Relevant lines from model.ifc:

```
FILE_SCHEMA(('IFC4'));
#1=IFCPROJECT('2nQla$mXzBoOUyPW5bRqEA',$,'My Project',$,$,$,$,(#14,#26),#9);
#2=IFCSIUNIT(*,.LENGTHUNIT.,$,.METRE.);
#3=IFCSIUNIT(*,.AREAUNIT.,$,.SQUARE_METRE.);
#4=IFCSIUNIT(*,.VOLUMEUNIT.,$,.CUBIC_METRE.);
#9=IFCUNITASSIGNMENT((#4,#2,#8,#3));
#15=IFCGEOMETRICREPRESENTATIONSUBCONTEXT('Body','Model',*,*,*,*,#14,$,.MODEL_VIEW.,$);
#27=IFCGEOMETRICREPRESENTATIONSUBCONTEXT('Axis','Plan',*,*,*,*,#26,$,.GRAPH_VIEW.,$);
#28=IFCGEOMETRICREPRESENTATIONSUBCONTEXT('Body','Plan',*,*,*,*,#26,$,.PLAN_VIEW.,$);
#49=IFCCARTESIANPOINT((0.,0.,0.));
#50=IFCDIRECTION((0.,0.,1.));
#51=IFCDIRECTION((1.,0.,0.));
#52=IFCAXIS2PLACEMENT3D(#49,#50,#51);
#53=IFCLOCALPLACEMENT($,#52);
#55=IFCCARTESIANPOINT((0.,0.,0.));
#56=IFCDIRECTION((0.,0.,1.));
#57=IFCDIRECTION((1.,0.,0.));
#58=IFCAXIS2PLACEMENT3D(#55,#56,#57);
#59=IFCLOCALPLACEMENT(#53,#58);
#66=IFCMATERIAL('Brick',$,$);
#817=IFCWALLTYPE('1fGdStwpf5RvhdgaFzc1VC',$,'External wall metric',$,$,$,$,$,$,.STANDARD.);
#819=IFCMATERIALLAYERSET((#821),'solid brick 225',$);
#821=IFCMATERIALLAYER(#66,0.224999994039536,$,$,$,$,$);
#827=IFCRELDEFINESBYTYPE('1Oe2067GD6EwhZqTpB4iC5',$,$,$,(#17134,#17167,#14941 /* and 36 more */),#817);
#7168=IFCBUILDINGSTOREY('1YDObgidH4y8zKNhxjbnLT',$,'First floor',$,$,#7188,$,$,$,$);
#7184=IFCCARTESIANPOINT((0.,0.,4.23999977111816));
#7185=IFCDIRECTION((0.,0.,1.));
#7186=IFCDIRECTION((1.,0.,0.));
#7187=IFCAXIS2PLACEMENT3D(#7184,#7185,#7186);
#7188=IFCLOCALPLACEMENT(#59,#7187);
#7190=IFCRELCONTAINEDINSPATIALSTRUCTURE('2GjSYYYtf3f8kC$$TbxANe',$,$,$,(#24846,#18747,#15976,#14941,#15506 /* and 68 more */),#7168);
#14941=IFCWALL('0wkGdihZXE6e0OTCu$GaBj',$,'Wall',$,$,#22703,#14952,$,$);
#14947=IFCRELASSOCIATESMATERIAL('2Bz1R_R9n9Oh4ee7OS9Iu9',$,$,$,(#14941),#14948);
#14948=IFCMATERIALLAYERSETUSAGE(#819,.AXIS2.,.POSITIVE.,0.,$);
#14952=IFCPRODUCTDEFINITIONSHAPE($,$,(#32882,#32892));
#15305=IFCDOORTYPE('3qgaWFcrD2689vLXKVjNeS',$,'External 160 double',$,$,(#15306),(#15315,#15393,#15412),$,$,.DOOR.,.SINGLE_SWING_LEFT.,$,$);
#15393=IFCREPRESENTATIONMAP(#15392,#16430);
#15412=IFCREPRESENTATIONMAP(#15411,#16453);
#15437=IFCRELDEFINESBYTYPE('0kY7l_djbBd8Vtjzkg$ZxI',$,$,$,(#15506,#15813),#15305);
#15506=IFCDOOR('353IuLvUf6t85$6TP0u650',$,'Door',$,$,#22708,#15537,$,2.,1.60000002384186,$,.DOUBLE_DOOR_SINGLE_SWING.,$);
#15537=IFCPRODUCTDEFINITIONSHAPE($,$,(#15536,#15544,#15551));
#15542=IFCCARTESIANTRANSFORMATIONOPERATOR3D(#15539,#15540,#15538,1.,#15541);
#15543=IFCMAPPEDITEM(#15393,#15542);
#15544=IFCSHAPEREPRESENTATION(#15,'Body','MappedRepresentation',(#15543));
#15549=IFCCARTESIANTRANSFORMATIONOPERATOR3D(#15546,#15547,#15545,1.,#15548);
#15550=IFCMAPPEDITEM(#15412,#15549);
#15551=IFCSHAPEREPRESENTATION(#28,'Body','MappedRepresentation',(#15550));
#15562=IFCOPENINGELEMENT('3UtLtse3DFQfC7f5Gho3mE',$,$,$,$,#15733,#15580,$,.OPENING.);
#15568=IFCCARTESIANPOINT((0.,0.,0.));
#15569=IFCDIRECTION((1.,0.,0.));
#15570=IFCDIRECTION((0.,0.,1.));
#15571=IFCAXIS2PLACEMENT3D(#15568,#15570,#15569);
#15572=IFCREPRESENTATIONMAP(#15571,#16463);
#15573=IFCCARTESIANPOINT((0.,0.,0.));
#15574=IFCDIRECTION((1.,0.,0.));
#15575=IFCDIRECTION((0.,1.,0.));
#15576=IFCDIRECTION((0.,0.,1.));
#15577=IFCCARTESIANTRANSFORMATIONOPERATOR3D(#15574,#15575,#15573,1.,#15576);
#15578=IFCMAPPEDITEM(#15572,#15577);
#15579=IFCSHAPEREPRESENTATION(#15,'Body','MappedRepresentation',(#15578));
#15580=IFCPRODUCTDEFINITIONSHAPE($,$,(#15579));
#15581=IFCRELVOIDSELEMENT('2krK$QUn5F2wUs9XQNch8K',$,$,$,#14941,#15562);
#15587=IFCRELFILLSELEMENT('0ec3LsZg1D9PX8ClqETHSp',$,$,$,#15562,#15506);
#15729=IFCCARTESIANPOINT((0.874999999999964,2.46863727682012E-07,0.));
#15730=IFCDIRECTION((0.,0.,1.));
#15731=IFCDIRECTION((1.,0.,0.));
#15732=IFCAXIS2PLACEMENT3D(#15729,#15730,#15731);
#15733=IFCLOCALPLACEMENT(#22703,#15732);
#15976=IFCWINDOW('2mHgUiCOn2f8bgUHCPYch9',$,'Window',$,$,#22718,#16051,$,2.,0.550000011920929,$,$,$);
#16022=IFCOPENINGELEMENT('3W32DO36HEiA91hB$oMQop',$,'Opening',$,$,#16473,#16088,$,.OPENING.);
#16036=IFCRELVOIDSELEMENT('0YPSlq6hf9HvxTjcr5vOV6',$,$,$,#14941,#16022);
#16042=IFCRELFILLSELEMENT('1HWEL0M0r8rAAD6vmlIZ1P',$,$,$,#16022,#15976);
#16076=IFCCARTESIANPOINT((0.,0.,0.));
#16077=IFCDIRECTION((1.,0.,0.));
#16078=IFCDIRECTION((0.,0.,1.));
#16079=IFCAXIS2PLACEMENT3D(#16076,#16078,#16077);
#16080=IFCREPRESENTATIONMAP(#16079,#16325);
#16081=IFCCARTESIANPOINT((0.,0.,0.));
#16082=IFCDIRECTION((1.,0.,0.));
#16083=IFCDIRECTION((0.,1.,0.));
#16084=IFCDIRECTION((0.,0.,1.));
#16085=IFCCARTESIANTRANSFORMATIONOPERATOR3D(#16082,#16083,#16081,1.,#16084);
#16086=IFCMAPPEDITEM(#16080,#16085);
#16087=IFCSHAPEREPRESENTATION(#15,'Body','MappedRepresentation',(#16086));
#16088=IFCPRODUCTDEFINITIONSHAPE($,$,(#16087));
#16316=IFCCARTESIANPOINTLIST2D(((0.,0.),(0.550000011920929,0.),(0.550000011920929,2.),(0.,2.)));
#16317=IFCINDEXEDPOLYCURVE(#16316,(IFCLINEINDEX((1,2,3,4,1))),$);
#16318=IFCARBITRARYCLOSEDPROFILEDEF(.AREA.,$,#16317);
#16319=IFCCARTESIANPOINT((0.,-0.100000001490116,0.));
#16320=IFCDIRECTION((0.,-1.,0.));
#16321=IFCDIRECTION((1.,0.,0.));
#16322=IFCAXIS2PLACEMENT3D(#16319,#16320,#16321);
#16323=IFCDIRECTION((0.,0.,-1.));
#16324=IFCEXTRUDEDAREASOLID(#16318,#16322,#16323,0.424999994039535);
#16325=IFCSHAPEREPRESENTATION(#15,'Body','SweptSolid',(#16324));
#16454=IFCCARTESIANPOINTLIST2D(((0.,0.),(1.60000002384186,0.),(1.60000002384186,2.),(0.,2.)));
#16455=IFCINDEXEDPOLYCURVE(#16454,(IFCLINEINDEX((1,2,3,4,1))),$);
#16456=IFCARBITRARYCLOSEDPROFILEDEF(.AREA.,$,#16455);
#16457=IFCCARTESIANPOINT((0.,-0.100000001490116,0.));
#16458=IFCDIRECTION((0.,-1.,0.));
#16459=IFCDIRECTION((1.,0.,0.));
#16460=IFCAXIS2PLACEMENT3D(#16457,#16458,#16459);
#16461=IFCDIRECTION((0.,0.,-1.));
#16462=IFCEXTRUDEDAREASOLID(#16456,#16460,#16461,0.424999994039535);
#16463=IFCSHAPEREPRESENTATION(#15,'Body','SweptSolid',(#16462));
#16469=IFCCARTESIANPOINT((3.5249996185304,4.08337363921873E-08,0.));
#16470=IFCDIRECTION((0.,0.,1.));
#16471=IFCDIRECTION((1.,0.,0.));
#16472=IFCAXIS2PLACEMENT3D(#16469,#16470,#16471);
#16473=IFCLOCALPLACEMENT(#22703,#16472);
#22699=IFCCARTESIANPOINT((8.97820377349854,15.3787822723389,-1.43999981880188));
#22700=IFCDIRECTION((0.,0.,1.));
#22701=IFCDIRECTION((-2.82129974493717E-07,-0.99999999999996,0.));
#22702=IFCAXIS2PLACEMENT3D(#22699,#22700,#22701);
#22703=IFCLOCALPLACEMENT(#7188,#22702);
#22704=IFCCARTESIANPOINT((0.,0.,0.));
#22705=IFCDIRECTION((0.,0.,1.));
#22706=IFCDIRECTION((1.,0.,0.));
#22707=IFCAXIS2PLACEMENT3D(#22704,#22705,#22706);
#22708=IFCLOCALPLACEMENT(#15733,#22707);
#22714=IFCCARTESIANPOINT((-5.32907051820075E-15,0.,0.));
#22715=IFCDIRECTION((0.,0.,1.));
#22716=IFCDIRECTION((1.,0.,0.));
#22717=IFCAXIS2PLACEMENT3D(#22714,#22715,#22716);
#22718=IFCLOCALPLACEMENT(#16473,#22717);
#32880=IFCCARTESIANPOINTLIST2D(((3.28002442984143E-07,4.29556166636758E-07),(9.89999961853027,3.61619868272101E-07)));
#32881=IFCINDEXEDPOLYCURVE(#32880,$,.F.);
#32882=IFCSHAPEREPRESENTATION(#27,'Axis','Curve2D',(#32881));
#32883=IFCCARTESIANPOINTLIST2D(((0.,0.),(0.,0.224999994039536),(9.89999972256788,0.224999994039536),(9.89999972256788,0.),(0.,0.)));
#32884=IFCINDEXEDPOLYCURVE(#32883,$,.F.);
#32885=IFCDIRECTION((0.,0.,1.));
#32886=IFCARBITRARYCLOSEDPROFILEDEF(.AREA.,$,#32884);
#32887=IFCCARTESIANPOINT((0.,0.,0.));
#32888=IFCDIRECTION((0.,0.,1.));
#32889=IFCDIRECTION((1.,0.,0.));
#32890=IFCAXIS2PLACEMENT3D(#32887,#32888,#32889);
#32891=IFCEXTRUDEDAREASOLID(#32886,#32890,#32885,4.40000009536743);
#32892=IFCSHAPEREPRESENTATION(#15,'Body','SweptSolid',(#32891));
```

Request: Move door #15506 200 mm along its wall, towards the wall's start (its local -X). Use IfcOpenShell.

```python
import ifcopenshell
import ifcopenshell.api.geometry
import ifcopenshell.util.placement

model = ifcopenshell.open("model.ifc")

door = model.by_id(15506)
opening = door.FillsVoids[0].RelatingOpeningElement
wall = opening.VoidsElements[0].RelatingBuildingElement

wall_matrix = ifcopenshell.util.placement.get_local_placement(wall.ObjectPlacement)
shift = wall_matrix[:3, 0] * -0.2
before = ifcopenshell.util.placement.get_local_placement(door.ObjectPlacement)[:3, 3].copy()

# The door is placed relative to its opening, so it follows when the opening moves.
matrix = ifcopenshell.util.placement.get_local_placement(opening.ObjectPlacement)
matrix[:3, 3] += shift
ifcopenshell.api.geometry.edit_object_placement(
    model, product=opening, matrix=matrix, is_si=False, should_transform_children=True
)

after = ifcopenshell.util.placement.get_local_placement(door.ObjectPlacement)[:3, 3]
print("door moved by", (after - before).round(3) + 0.0)

model.write("model_v2.ifc")
```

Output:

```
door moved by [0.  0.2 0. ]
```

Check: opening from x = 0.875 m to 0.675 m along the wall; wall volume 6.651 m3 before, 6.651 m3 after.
